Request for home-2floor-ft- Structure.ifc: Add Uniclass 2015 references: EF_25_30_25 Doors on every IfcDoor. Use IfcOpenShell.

First a look at what the model holds.

```python
import ifcopenshell

model = ifcopenshell.open("home-2floor-ft- Structure.ifc")
print(model.schema)
print("classifications:", [c.Name for c in model.by_type("IfcClassification")])
for ifc_class in ("IfcDoor", "IfcRoof", "IfcStair", "IfcWall", "IfcWindow"):
    print(ifc_class, len(model.by_type(ifc_class)))
```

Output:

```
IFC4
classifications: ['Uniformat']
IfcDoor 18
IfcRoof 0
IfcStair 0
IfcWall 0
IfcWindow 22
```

```python
import ifcopenshell
import ifcopenshell.api.classification

model = ifcopenshell.open("home-2floor-ft- Structure.ifc")

system = ifcopenshell.api.classification.add_classification(model, classification="Uniclass 2015")

codes = {
    "IfcDoor": ("EF_25_30_25", "Doors"),
}
for ifc_class, (code, name) in codes.items():
    products = model.by_type(ifc_class)
    ifcopenshell.api.classification.add_reference(
        model, products=products, classification=system, identification=code, name=name
    )
    print(code, len(products))

model.write("home-2floor-ft- Structure_rev.ifc")
```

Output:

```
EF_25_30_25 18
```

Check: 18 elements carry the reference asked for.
